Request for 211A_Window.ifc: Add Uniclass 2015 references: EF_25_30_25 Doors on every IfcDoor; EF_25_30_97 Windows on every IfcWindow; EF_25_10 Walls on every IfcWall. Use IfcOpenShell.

First a look at what the model holds.

```python
import ifcopenshell

model = ifcopenshell.open("211A_Window.ifc")
print(model.schema)
print("classifications:", [c.Name for c in model.by_type("IfcClassification")])
for ifc_class in ("IfcDoor", "IfcRoof", "IfcStair", "IfcWall", "IfcWindow"):
    print(ifc_class, len(model.by_type(ifc_class)))
```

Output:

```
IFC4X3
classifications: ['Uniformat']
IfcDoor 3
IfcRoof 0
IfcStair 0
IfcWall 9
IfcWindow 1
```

```python
import ifcopenshell
import ifcopenshell.api.classification

model = ifcopenshell.open("211A_Window.ifc")

system = ifcopenshell.api.classification.add_classification(model, classification="Uniclass 2015")

codes = {
    "IfcDoor": ("EF_25_30_25", "Doors"),
    "IfcWindow": ("EF_25_30_97", "Windows"),
    "IfcWall": ("EF_25_10", "Walls"),
}
for ifc_class, (code, name) in codes.items():
    products = model.by_type(ifc_class)
    ifcopenshell.api.classification.add_reference(
        model, products=products, classification=system, identification=code, name=name
    )
    print(code, len(products))

model.write("211A_Window_v2.ifc")
```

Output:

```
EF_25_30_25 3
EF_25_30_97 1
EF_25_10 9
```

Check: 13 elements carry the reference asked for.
